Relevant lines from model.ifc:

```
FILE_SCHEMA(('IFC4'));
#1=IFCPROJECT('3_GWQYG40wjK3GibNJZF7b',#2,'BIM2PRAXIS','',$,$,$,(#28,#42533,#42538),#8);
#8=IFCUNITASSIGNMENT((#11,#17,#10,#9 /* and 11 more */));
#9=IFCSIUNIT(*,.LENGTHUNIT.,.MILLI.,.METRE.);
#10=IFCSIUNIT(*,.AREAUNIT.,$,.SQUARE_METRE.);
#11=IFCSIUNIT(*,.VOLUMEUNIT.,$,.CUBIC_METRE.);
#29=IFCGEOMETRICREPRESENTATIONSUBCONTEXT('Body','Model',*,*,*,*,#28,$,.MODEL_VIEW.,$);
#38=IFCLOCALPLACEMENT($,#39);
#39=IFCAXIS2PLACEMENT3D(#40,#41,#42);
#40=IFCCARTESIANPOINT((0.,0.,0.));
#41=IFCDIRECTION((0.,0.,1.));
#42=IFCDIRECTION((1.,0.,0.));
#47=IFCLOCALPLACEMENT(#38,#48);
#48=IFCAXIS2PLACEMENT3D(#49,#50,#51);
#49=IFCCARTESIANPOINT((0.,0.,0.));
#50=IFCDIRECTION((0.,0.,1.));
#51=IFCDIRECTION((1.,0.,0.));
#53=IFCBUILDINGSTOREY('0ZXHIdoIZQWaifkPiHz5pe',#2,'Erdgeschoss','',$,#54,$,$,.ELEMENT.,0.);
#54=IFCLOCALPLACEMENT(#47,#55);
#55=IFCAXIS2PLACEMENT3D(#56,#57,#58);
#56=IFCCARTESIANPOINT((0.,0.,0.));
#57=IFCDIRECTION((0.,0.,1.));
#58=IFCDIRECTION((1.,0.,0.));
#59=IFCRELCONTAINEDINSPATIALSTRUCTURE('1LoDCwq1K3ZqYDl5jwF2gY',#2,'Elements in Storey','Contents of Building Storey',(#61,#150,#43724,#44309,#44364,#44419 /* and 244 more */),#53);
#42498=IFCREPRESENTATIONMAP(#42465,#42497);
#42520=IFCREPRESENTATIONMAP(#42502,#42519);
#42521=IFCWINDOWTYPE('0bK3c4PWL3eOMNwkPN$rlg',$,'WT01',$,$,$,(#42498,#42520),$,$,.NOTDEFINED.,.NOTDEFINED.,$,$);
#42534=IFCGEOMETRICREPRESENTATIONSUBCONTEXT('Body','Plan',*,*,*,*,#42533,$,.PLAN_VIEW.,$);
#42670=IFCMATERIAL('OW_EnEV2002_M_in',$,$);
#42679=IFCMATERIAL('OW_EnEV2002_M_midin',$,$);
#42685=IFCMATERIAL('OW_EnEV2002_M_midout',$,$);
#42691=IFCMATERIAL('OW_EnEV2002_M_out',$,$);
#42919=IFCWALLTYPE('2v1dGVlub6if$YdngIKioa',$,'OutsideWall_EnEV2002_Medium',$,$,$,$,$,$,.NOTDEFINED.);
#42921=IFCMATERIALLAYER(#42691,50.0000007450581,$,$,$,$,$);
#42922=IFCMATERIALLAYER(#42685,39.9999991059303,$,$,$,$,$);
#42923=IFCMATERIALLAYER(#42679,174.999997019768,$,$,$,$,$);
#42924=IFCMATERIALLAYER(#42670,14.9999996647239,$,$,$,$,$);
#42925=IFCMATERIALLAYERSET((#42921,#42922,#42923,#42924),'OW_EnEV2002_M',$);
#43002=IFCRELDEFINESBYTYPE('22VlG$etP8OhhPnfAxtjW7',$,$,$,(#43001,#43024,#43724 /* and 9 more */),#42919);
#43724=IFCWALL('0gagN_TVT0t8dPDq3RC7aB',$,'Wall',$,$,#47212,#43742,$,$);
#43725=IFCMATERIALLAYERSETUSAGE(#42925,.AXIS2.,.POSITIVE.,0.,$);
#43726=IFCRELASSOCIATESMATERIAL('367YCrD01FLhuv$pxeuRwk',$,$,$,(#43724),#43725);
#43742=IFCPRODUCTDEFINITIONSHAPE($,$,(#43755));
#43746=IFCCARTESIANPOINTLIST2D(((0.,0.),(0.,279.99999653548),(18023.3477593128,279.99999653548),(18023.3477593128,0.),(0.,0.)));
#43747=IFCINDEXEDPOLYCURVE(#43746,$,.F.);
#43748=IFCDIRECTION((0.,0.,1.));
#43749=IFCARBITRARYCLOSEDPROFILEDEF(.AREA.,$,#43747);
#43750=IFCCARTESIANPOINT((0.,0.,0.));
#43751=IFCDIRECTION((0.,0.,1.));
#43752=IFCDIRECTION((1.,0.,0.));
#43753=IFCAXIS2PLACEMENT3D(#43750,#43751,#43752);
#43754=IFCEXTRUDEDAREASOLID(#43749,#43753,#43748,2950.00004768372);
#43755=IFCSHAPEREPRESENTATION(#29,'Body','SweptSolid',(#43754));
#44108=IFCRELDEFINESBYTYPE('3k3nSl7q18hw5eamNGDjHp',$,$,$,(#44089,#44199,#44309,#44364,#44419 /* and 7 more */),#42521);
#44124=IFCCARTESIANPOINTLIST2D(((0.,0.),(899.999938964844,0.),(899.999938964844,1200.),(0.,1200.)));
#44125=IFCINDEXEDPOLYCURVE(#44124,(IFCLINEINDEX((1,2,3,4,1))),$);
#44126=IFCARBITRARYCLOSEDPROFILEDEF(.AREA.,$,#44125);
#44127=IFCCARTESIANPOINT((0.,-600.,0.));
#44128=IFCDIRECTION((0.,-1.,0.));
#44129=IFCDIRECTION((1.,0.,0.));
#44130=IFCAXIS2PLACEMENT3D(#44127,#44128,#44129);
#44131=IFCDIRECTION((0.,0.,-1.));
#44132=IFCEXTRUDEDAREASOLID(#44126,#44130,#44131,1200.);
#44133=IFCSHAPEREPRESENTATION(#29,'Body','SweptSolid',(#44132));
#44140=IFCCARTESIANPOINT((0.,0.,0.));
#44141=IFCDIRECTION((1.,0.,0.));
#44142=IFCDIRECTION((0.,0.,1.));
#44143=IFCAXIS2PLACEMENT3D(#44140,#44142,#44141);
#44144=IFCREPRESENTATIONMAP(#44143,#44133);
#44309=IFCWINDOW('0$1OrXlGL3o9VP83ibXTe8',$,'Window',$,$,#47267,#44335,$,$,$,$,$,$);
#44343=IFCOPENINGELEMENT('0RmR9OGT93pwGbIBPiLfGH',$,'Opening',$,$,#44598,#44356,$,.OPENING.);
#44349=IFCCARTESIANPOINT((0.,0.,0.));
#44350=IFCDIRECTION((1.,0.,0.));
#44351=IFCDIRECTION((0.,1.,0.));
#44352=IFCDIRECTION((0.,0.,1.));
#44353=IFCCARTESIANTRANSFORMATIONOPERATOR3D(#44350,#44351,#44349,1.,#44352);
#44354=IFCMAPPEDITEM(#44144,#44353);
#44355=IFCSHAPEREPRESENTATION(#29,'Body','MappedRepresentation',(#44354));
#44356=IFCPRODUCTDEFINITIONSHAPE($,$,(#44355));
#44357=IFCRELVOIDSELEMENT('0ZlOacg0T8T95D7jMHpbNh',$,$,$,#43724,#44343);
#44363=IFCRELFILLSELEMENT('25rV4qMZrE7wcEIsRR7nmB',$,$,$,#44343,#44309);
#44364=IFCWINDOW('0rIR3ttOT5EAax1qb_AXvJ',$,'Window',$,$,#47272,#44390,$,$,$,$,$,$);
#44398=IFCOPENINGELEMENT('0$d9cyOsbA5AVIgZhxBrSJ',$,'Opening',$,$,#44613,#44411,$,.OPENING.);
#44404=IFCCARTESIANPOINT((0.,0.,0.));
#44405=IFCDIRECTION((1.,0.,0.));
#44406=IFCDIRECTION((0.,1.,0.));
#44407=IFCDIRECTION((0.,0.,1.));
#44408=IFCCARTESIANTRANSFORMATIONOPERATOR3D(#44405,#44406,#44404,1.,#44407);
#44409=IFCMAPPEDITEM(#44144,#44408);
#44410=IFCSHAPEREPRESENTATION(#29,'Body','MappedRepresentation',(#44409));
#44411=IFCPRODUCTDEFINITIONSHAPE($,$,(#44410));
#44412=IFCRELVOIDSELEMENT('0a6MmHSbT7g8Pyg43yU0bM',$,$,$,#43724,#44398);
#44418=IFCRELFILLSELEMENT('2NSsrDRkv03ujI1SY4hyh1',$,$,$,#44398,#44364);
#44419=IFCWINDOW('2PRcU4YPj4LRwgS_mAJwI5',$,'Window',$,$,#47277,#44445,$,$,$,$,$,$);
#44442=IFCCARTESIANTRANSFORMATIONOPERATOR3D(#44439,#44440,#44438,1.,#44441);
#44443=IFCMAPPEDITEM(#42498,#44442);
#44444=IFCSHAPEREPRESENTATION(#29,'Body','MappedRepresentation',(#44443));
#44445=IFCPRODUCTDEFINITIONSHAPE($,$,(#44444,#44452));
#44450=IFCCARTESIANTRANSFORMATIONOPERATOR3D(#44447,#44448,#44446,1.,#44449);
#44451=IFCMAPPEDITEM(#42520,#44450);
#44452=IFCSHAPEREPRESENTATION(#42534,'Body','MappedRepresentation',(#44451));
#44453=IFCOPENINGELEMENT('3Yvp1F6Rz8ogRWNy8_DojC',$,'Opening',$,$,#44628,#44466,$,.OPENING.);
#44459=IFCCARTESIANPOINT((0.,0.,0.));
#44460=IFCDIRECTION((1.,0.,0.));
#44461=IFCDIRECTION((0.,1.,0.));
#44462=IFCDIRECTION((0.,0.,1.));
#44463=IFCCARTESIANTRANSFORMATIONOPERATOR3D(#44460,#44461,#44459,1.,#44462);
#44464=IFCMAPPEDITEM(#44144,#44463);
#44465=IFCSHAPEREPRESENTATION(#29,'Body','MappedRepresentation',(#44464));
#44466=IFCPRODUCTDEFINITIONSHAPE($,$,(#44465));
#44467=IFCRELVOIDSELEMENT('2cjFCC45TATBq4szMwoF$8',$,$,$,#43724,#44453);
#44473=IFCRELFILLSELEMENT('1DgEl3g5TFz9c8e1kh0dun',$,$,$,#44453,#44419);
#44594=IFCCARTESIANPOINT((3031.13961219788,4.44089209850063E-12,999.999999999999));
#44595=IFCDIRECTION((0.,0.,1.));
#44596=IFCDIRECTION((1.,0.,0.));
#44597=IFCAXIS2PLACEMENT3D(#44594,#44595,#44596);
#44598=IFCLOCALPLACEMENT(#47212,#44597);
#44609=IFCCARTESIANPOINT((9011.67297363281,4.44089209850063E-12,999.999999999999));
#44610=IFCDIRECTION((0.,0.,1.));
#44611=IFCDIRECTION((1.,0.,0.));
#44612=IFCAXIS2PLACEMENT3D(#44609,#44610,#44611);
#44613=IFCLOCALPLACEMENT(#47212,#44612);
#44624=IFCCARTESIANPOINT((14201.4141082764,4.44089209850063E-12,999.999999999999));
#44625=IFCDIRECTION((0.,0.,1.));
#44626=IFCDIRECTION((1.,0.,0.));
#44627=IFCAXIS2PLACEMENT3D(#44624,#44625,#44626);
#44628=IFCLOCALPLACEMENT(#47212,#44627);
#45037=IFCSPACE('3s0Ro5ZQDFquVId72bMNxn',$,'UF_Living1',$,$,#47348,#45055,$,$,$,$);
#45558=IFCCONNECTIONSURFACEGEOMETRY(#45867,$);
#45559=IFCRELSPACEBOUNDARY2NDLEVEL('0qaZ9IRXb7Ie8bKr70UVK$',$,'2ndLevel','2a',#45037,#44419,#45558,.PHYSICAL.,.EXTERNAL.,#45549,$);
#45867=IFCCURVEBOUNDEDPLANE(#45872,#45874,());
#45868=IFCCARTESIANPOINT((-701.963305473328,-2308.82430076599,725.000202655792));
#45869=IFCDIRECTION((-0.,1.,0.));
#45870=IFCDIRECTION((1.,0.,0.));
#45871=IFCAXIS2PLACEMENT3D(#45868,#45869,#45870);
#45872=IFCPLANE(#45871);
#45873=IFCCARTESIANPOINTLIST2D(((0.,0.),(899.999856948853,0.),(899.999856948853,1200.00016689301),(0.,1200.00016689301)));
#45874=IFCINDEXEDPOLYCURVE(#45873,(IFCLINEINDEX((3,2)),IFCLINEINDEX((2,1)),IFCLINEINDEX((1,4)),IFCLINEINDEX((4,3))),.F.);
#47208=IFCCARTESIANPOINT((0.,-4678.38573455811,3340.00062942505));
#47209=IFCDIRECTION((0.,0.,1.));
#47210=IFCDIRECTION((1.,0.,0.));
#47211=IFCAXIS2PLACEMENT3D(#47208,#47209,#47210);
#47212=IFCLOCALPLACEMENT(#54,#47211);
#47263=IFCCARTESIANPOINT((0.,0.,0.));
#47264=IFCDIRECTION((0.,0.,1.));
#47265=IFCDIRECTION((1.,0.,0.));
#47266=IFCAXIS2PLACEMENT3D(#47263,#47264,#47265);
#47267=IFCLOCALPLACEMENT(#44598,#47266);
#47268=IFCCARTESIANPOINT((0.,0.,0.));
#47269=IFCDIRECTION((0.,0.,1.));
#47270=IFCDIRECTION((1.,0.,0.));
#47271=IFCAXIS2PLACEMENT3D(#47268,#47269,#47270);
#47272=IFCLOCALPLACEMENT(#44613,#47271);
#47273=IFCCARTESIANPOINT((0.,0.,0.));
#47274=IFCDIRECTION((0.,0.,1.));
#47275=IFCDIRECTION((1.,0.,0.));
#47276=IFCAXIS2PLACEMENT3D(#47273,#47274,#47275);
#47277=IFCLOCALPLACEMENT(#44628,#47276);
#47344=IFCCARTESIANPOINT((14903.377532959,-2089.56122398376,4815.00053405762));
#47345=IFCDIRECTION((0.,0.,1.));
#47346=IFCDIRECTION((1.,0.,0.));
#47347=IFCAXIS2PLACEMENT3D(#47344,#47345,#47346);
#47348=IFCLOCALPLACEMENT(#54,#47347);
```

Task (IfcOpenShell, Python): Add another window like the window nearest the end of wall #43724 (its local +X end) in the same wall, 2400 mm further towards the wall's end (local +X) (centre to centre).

```python
import numpy as np
import ifcopenshell
import ifcopenshell.api.feature
import ifcopenshell.api.geometry
import ifcopenshell.api.root
import ifcopenshell.geom
import ifcopenshell.util.element
import ifcopenshell.util.placement
import ifcopenshell.util.shape
import ifcopenshell.util.unit

model = ifcopenshell.open("model.ifc")
unit_scale = ifcopenshell.util.unit.calculate_unit_scale(model)
settings = ifcopenshell.geom.settings()


def volume(element):
    """Net volume in cubic metres, openings subtracted."""
    shape = ifcopenshell.geom.create_shape(settings, element)
    return ifcopenshell.util.shape.get_volume(shape.geometry)


window = model.by_id(44419)
opening = window.FillsVoids[0].RelatingOpeningElement
wall = opening.VoidsElements[0].RelatingBuildingElement
before = volume(wall)
shift = ifcopenshell.util.placement.get_local_placement(wall.ObjectPlacement)[:3, 0] * 2.4 / unit_scale

# copy_class copies the void relationship, type, container and properties, but no geometry.
new_opening = ifcopenshell.api.root.copy_class(model, product=opening)
new_opening.Representation = ifcopenshell.util.element.copy_deep(
    model, opening.Representation, exclude=["IfcGeometricRepresentationContext", "IfcRepresentationMap"]
)
new_window = ifcopenshell.api.root.copy_class(model, product=window)
new_window.Representation = ifcopenshell.util.element.copy_deep(
    model, window.Representation, exclude=["IfcGeometricRepresentationContext", "IfcRepresentationMap"]
)
ifcopenshell.api.feature.add_filling(model, opening=new_opening, element=new_window)

for old, new in ((opening, new_opening), (window, new_window)):
    matrix = ifcopenshell.util.placement.get_local_placement(old.ObjectPlacement)
    matrix[:3, 3] += shift
    ifcopenshell.api.geometry.edit_object_placement(model, product=new, matrix=matrix, is_si=False)

# The copied space boundaries still share their surfaces with the original.
for rel in new_window.ProvidesBoundaries:
    if rel.ConnectionGeometry:
        rel.ConnectionGeometry = ifcopenshell.util.element.copy_deep(model, rel.ConnectionGeometry)

# Space boundary surfaces are stored in each space's coordinates; move them too.
for rel in new_window.ProvidesBoundaries:
    if not rel.ConnectionGeometry:
        continue
    surface = rel.ConnectionGeometry.SurfaceOnRelatingElement.BasisSurface
    space_matrix = ifcopenshell.util.placement.get_local_placement(rel.RelatingSpace.ObjectPlacement)
    point = np.array(surface.Position.Location.Coordinates) + space_matrix[:3, :3].T @ shift
    surface.Position = model.createIfcAxis2Placement3D(
        model.createIfcCartesianPoint(point.tolist()), surface.Position.Axis, surface.Position.RefDirection
    )

after = volume(wall)

print(f"wall volume {before:.3f} -> {after:.3f} m3")

model.write("model_edited.ifc")
```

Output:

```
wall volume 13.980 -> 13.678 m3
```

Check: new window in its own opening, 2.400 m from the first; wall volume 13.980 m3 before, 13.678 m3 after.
